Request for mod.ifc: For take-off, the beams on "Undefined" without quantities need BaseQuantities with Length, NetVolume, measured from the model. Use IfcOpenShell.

First a look at what the model holds.

```python
import ifcopenshell
import ifcopenshell.util.element
import ifcopenshell.util.unit

model = ifcopenshell.open("mod.ifc")
print(model.schema)
for unit_type in ("LENGTHUNIT", "AREAUNIT", "VOLUMEUNIT"):
    print(unit_type, ifcopenshell.util.unit.calculate_unit_scale(model, unit_type))
storey = next(s for s in model.by_type("IfcBuildingStorey") if s.Name == "Undefined")
beams = [e for e in ifcopenshell.util.element.get_decomposition(storey) if e.is_a("IfcBeam")]
for e in sorted(beams, key=lambda e: e.id()):
    print(e.id(), e.is_a(), e.Name, list(ifcopenshell.util.element.get_psets(e, qtos_only=True)), sep=" | ")
```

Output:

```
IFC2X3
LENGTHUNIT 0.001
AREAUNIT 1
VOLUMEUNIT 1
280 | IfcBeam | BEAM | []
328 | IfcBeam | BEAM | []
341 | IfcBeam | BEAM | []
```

```python
import ifcopenshell
import ifcopenshell.api.pset
import ifcopenshell.geom
import ifcopenshell.util.element
import ifcopenshell.util.shape
import ifcopenshell.util.unit

model = ifcopenshell.open("mod.ifc")
unit_scale = ifcopenshell.util.unit.calculate_unit_scale(model)
volume_scale = ifcopenshell.util.unit.calculate_unit_scale(model, "VOLUMEUNIT")
settings = ifcopenshell.geom.settings()

storey = next(s for s in model.by_type("IfcBuildingStorey") if s.Name == "Undefined")
beams = [e for e in ifcopenshell.util.element.get_decomposition(storey) if e.is_a("IfcBeam")]

for e in sorted(beams, key=lambda e: e.id()):
    if ifcopenshell.util.element.get_psets(e, qtos_only=True, should_inherit=False):
        continue
    # Geometry comes back in metres, in the element's own axes.
    shape = ifcopenshell.geom.create_shape(settings, e)
    values = {
        "Length": ifcopenshell.util.shape.get_max_xyz(shape.geometry) / unit_scale,
        "NetVolume": ifcopenshell.util.shape.get_volume(shape.geometry) / volume_scale,
    }
    qto = ifcopenshell.api.pset.add_qto(model, product=e, name="BaseQuantities")
    ifcopenshell.api.pset.edit_qto(model, qto=qto, properties=values)
    print(e.id(), {k: round(v, 3) for k, v in values.items()})

model.write("mod_rev.ifc")
```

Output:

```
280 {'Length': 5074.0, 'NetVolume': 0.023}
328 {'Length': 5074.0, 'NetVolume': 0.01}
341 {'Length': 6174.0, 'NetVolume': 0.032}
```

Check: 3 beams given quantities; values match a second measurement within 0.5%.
